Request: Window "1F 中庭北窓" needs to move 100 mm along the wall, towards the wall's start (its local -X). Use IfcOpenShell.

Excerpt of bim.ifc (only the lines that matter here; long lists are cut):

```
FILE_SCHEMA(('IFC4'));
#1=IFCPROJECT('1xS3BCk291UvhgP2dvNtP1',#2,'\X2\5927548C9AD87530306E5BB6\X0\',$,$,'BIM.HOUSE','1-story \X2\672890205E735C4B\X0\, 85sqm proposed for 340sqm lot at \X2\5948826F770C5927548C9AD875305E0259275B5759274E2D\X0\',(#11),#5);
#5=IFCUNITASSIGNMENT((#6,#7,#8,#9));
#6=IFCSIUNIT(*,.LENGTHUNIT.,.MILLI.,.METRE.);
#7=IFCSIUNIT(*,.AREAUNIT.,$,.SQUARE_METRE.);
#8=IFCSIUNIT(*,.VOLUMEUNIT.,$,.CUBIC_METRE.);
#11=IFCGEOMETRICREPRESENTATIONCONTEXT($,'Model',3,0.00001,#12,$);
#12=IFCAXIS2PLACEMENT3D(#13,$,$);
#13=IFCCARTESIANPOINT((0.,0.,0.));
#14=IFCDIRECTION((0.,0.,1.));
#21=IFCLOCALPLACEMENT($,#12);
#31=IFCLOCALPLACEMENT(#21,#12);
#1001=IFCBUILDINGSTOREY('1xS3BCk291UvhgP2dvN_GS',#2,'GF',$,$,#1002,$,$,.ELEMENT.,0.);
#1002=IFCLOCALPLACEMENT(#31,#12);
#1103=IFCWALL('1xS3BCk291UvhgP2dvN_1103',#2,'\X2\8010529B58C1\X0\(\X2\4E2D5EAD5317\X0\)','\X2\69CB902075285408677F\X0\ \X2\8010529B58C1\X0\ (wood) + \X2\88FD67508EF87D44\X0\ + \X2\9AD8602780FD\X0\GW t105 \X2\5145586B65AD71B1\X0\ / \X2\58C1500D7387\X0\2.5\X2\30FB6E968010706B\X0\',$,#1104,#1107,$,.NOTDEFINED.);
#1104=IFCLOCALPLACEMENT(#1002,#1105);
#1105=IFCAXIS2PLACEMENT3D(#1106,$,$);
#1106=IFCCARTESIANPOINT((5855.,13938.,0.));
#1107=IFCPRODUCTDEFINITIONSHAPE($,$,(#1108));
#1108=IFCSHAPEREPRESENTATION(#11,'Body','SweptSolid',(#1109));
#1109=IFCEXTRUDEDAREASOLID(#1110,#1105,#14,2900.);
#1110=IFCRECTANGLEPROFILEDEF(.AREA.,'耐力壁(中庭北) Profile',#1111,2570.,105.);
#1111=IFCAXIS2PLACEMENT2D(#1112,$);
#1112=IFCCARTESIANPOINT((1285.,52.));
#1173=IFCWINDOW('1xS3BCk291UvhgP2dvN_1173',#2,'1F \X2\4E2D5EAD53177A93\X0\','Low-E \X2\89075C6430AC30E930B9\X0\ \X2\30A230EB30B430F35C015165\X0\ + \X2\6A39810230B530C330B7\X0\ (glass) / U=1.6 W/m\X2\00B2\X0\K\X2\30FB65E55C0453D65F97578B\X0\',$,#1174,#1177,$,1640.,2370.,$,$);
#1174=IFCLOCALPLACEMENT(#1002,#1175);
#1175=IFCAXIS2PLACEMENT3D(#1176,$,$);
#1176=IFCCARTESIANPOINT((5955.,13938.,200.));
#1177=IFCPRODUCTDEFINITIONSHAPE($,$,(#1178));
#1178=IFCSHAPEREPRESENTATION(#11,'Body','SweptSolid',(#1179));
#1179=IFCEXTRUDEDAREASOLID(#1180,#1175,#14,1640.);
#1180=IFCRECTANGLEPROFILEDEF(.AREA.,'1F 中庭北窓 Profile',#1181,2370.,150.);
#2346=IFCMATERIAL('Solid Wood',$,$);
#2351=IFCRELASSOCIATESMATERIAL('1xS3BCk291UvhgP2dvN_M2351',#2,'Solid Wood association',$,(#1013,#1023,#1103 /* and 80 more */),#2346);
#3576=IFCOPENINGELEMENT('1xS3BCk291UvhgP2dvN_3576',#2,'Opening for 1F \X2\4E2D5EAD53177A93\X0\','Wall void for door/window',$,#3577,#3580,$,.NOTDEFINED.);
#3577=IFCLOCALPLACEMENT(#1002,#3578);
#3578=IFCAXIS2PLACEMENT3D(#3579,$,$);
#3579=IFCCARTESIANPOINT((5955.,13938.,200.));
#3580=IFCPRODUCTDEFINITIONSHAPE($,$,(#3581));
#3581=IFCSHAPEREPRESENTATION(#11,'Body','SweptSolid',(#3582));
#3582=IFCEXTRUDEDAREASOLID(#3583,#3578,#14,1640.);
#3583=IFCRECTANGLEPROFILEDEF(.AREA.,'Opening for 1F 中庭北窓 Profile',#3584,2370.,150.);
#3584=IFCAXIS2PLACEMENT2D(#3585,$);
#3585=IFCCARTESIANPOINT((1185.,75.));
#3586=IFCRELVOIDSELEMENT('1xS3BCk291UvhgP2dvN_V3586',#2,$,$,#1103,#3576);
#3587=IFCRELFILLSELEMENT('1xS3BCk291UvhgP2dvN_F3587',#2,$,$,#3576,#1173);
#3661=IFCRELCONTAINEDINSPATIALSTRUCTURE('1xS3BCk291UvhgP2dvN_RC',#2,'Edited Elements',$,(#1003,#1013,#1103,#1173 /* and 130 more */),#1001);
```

```python
import ifcopenshell
import ifcopenshell.api.geometry
import ifcopenshell.util.placement
import ifcopenshell.util.unit

model = ifcopenshell.open("bim.ifc")
unit_scale = ifcopenshell.util.unit.calculate_unit_scale(model)

window = model.by_guid("1xS3BCk291UvhgP2dvN_1173")
opening = window.FillsVoids[0].RelatingOpeningElement
wall = opening.VoidsElements[0].RelatingBuildingElement

wall_matrix = ifcopenshell.util.placement.get_local_placement(wall.ObjectPlacement)
shift = wall_matrix[:3, 0] * -0.1 / unit_scale
before = ifcopenshell.util.placement.get_local_placement(window.ObjectPlacement)[:3, 3].copy()

# The window is not placed relative to its opening, so move both.
for product in (opening, window):
    matrix = ifcopenshell.util.placement.get_local_placement(product.ObjectPlacement)
    matrix[:3, 3] += shift
    ifcopenshell.api.geometry.edit_object_placement(model, product=product, matrix=matrix, is_si=False)

after = ifcopenshell.util.placement.get_local_placement(window.ObjectPlacement)[:3, 3]
print("window moved by", (after - before).round(3) + 0.0)

model.write("bim_rev.ifc")
```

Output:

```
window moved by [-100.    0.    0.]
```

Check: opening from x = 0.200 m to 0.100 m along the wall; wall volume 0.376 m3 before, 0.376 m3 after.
